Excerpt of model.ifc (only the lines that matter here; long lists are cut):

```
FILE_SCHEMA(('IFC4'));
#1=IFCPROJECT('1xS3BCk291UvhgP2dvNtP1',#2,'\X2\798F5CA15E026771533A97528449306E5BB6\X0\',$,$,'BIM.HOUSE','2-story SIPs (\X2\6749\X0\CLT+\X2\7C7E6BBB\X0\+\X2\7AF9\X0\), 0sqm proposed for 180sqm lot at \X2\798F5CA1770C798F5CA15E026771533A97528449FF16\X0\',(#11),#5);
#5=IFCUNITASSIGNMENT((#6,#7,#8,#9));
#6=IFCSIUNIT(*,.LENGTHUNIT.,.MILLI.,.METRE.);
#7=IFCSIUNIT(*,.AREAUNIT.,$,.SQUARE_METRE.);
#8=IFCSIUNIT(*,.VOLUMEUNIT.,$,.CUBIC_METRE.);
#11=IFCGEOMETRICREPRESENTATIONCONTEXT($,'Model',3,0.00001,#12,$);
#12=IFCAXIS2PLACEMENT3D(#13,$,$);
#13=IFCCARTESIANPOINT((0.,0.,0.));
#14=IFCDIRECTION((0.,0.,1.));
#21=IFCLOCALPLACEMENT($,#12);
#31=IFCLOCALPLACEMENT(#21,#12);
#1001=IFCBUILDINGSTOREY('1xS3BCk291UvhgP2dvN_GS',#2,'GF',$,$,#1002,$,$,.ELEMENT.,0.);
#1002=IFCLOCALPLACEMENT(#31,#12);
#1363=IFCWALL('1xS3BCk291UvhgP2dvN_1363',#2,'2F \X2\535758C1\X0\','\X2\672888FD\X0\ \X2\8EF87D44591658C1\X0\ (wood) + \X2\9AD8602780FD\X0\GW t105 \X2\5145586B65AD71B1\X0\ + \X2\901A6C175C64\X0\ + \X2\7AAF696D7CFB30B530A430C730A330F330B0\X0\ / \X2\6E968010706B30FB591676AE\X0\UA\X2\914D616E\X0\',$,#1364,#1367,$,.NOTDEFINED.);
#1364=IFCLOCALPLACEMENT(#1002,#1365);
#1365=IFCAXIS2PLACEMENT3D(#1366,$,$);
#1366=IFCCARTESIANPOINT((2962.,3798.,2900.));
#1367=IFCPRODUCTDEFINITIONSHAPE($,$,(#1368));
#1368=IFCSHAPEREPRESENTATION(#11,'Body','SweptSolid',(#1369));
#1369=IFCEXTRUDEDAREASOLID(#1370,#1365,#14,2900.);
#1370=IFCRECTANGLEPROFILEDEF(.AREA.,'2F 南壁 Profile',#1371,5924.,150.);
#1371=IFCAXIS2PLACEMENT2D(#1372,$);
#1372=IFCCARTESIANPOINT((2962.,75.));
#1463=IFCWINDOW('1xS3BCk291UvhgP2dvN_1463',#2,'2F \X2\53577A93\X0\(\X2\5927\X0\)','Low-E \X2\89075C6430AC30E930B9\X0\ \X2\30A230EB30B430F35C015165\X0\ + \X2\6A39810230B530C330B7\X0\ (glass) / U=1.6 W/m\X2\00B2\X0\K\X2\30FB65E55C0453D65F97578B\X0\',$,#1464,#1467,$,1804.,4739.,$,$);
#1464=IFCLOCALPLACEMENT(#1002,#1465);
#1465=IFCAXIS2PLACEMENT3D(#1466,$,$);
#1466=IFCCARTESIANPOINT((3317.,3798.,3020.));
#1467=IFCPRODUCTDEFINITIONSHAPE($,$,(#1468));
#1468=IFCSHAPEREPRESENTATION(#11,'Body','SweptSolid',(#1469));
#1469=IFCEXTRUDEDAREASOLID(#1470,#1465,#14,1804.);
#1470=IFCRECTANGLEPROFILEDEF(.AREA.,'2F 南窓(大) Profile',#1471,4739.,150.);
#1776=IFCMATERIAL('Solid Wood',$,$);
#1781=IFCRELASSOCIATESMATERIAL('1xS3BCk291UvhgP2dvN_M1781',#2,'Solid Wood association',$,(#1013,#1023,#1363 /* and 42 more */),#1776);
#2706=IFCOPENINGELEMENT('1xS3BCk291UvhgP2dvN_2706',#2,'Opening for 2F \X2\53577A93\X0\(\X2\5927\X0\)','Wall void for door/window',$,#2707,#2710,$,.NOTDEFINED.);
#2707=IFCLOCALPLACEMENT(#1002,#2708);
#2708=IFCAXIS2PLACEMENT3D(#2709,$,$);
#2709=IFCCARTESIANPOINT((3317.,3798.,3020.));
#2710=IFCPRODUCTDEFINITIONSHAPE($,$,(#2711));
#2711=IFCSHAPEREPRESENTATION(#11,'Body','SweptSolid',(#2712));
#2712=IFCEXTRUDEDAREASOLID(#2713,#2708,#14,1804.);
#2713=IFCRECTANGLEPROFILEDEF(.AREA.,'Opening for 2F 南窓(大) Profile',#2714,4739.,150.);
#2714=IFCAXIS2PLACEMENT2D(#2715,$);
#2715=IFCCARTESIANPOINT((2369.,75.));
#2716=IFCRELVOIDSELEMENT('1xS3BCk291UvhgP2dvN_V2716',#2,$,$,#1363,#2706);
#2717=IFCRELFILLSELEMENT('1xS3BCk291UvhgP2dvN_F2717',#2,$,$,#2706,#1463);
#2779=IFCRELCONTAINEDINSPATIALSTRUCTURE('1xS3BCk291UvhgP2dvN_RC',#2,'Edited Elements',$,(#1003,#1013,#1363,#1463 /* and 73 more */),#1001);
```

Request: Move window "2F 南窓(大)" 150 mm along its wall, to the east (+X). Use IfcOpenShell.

```python
import ifcopenshell
import ifcopenshell.api.geometry
import ifcopenshell.util.placement

model = ifcopenshell.open("model.ifc")

window = model.by_guid("1xS3BCk291UvhgP2dvN_1463")
opening = window.FillsVoids[0].RelatingOpeningElement
wall = opening.VoidsElements[0].RelatingBuildingElement

wall_matrix = ifcopenshell.util.placement.get_local_placement(wall.ObjectPlacement)
shift = wall_matrix[:3, 0] * 150.0
before = ifcopenshell.util.placement.get_local_placement(window.ObjectPlacement)[:3, 3].copy()

# The window is not placed relative to its opening, so move both.
for product in (opening, window):
    matrix = ifcopenshell.util.placement.get_local_placement(product.ObjectPlacement)
    matrix[:3, 3] += shift
    ifcopenshell.api.geometry.edit_object_placement(model, product=product, matrix=matrix, is_si=False)

after = ifcopenshell.util.placement.get_local_placement(window.ObjectPlacement)[:3, 3]
print("window moved by", (after - before).round(3) + 0.0)

model.write("model_edited.ifc")
```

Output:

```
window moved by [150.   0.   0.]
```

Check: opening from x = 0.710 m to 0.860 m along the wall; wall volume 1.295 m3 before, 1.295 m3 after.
